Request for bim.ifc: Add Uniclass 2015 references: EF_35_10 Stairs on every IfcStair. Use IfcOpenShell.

First a look at what the model holds.

```python
import ifcopenshell

model = ifcopenshell.open("bim.ifc")
print(model.schema)
print("classifications:", [c.Name for c in model.by_type("IfcClassification")])
for ifc_class in ("IfcDoor", "IfcRoof", "IfcStair", "IfcWall", "IfcWindow"):
    print(ifc_class, len(model.by_type(ifc_class)))
```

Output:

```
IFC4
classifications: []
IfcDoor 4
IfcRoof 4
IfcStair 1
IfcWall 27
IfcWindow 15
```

```python
import ifcopenshell
import ifcopenshell.api.classification

model = ifcopenshell.open("bim.ifc")

system = ifcopenshell.api.classification.add_classification(model, classification="Uniclass 2015")

codes = {
    "IfcStair": ("EF_35_10", "Stairs"),
}
for ifc_class, (code, name) in codes.items():
    products = model.by_type(ifc_class)
    ifcopenshell.api.classification.add_reference(
        model, products=products, classification=system, identification=code, name=name
    )
    print(code, len(products))

model.write("bim_edited.ifc")
```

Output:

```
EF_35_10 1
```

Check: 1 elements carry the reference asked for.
